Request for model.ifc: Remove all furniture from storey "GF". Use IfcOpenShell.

First a look at what the model holds.

```python
import ifcopenshell
import ifcopenshell.util.element

model = ifcopenshell.open("model.ifc")
print(model.schema)
storey = next(s for s in model.by_type("IfcBuildingStorey") if s.Name == "GF")
furniture = [e for e in ifcopenshell.util.element.get_decomposition(storey) if e.is_a("IfcFurnishingElement")]
seen = {}
for e in furniture:
    element_type = ifcopenshell.util.element.get_type(e)
    name = element_type.Name if element_type not in (None, e) else None
    seen[name] = seen.get(name, 0) + 1
for name, count in sorted(seen.items(), key=str):
    print(count, "x", name)
```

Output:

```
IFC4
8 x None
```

```python
import ifcopenshell
import ifcopenshell.api.root
import ifcopenshell.util.element

model = ifcopenshell.open("model.ifc")

storey = next(s for s in model.by_type("IfcBuildingStorey") if s.Name == "GF")
furniture = [e for e in ifcopenshell.util.element.get_decomposition(storey) if e.is_a("IfcFurnishingElement")]

for e in furniture:
    ifcopenshell.api.root.remove_product(model, product=e)
print(len(furniture), "removed")

model.write("model_rev.ifc")
```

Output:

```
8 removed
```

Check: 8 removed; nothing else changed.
